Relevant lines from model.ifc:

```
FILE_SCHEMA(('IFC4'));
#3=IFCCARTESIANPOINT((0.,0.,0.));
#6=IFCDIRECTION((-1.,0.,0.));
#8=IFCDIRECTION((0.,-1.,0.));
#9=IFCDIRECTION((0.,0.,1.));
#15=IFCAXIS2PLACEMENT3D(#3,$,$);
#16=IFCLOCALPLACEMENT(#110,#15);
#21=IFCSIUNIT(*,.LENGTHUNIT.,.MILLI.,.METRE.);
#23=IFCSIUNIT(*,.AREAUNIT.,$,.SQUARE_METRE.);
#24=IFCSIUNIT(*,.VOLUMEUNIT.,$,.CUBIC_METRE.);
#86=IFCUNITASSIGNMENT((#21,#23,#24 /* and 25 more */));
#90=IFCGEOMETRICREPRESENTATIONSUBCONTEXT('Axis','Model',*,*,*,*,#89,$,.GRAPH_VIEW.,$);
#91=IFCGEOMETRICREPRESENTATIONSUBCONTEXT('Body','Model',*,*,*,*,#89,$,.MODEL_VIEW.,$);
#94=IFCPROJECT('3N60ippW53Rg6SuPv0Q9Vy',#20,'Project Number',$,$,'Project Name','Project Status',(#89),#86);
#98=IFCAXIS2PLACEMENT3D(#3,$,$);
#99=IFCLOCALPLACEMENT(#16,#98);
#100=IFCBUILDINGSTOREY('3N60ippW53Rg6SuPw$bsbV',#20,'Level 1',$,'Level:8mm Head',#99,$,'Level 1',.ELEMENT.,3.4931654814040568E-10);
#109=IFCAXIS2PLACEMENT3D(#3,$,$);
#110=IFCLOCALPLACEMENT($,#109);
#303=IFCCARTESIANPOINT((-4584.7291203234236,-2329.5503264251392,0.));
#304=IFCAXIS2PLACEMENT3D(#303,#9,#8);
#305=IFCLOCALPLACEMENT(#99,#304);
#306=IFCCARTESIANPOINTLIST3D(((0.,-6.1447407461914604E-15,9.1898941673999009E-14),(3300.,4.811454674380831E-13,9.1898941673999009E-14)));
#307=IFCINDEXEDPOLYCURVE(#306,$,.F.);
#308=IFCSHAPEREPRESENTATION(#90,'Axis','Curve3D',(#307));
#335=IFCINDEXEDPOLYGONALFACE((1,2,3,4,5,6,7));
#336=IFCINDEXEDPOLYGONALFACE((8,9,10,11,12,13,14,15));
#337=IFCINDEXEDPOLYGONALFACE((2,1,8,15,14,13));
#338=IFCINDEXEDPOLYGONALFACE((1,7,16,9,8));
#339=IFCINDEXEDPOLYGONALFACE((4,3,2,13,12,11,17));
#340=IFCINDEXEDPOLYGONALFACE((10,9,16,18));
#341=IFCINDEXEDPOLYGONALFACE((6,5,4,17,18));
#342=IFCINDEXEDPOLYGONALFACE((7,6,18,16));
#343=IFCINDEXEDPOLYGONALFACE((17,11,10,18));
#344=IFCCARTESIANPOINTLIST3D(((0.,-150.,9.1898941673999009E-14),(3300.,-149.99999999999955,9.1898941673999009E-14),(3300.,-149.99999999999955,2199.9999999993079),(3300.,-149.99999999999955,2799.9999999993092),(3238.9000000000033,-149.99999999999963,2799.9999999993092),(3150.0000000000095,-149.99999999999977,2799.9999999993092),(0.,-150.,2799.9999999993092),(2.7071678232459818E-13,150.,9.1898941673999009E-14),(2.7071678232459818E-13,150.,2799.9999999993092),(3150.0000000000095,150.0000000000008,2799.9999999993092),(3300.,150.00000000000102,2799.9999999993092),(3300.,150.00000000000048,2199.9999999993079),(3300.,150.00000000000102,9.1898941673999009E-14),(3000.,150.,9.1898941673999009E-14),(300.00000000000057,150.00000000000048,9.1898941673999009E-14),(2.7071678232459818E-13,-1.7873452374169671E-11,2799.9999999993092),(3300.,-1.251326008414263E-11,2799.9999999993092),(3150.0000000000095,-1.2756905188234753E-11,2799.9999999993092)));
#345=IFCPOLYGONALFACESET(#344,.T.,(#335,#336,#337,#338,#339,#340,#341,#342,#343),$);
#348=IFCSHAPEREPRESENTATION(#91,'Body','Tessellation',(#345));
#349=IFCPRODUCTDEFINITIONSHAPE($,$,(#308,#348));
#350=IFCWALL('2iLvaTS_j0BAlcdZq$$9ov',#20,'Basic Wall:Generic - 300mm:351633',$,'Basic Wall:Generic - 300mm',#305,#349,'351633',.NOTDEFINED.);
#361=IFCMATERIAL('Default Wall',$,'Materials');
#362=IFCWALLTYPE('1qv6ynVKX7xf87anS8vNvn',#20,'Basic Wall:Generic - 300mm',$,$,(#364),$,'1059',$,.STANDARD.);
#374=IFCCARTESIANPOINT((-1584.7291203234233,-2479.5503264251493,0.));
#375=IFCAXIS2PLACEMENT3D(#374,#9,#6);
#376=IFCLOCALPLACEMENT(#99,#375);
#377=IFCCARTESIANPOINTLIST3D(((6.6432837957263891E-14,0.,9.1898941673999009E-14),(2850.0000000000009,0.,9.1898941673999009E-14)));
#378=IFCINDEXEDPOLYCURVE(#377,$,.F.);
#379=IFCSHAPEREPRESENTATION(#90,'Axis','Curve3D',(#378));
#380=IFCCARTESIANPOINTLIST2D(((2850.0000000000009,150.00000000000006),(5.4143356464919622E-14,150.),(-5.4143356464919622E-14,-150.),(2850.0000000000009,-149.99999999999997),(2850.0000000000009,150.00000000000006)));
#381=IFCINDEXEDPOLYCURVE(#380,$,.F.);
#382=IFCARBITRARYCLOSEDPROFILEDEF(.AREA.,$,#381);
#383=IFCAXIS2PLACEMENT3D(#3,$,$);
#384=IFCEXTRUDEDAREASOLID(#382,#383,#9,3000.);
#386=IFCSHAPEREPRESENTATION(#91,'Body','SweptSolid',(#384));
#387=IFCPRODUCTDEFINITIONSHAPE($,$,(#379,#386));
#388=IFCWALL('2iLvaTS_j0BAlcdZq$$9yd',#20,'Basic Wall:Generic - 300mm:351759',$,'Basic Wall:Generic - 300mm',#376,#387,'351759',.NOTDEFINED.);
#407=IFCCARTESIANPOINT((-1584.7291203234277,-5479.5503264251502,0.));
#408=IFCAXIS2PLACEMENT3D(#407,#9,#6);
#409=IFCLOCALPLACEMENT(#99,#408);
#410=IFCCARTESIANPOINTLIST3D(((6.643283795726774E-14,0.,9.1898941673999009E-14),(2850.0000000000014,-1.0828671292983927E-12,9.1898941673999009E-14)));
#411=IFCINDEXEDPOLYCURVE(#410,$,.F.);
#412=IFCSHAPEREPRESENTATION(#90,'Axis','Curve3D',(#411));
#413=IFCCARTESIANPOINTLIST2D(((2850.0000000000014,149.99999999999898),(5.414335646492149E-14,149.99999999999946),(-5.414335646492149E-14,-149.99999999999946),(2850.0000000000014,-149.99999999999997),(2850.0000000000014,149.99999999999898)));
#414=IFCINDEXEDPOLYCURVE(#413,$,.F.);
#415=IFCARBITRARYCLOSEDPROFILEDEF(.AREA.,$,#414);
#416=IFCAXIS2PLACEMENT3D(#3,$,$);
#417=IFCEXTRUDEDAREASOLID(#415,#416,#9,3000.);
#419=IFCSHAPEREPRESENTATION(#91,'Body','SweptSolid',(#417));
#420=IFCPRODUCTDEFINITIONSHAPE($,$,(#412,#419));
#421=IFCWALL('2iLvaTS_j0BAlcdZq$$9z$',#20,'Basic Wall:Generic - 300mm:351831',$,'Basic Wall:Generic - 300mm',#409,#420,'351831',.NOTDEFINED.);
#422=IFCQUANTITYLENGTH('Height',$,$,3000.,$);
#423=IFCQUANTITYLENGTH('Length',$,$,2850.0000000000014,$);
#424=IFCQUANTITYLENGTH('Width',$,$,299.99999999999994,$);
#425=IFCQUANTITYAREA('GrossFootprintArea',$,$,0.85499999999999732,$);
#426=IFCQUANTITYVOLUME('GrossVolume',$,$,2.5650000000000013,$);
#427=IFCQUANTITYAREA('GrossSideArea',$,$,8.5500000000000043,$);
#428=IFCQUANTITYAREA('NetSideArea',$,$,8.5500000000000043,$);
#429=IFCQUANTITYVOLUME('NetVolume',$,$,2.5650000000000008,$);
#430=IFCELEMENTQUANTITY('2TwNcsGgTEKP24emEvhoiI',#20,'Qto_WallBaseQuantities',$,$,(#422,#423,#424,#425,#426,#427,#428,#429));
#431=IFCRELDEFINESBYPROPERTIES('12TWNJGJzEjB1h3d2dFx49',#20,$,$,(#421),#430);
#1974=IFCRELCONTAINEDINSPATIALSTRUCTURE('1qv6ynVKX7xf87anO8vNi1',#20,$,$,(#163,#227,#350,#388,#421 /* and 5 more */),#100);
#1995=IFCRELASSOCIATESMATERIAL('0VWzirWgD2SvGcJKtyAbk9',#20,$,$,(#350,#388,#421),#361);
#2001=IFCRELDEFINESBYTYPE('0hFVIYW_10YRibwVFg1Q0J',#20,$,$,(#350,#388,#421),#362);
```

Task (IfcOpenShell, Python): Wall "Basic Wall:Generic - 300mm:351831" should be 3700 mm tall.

```python
import ifcopenshell
import ifcopenshell.api.pset
import ifcopenshell.geom
import ifcopenshell.util.element
import ifcopenshell.util.representation
import ifcopenshell.util.shape
import ifcopenshell.util.unit

model = ifcopenshell.open("model.ifc")
unit_scale = ifcopenshell.util.unit.calculate_unit_scale(model)
area_scale = ifcopenshell.util.unit.calculate_unit_scale(model, "AREAUNIT")
volume_scale = ifcopenshell.util.unit.calculate_unit_scale(model, "VOLUMEUNIT")
settings = ifcopenshell.geom.settings()


def volume(element):
    """Net volume in cubic metres, openings subtracted."""
    shape = ifcopenshell.geom.create_shape(settings, element)
    return ifcopenshell.util.shape.get_volume(shape.geometry)


wall = model.by_guid("2iLvaTS_j0BAlcdZq$$9z$")
before = volume(wall)

body = ifcopenshell.util.representation.get_representation(wall, "Model", "Body")
solid = body.Items[0]
old_height = solid.Depth
solid.Depth = 3.7 / unit_scale
after = volume(wall)
thickness = 0.3  # wall thickness in metres

# Update the stored height, areas and volumes.
qto = model.by_id(ifcopenshell.util.element.get_pset(wall, "Qto_WallBaseQuantities", should_inherit=False)["id"])
ifcopenshell.api.pset.edit_qto(model, qto=qto, properties={
    "Height": solid.Depth,
    "GrossVolume": ifcopenshell.util.element.get_pset(wall, "Qto_WallBaseQuantities", "GrossVolume") * solid.Depth / old_height,
    "GrossSideArea": ifcopenshell.util.element.get_pset(wall, "Qto_WallBaseQuantities", "GrossSideArea") * solid.Depth / old_height,
    "NetSideArea": after / thickness / area_scale,
    "NetVolume": after / volume_scale,
})

print(f"height {old_height:g} -> {solid.Depth:g}, volume {before:.3f} -> {after:.3f} m3")

model.write("model_updated.ifc")
```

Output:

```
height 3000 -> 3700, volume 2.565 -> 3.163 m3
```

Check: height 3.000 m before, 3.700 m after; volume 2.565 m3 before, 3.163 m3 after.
